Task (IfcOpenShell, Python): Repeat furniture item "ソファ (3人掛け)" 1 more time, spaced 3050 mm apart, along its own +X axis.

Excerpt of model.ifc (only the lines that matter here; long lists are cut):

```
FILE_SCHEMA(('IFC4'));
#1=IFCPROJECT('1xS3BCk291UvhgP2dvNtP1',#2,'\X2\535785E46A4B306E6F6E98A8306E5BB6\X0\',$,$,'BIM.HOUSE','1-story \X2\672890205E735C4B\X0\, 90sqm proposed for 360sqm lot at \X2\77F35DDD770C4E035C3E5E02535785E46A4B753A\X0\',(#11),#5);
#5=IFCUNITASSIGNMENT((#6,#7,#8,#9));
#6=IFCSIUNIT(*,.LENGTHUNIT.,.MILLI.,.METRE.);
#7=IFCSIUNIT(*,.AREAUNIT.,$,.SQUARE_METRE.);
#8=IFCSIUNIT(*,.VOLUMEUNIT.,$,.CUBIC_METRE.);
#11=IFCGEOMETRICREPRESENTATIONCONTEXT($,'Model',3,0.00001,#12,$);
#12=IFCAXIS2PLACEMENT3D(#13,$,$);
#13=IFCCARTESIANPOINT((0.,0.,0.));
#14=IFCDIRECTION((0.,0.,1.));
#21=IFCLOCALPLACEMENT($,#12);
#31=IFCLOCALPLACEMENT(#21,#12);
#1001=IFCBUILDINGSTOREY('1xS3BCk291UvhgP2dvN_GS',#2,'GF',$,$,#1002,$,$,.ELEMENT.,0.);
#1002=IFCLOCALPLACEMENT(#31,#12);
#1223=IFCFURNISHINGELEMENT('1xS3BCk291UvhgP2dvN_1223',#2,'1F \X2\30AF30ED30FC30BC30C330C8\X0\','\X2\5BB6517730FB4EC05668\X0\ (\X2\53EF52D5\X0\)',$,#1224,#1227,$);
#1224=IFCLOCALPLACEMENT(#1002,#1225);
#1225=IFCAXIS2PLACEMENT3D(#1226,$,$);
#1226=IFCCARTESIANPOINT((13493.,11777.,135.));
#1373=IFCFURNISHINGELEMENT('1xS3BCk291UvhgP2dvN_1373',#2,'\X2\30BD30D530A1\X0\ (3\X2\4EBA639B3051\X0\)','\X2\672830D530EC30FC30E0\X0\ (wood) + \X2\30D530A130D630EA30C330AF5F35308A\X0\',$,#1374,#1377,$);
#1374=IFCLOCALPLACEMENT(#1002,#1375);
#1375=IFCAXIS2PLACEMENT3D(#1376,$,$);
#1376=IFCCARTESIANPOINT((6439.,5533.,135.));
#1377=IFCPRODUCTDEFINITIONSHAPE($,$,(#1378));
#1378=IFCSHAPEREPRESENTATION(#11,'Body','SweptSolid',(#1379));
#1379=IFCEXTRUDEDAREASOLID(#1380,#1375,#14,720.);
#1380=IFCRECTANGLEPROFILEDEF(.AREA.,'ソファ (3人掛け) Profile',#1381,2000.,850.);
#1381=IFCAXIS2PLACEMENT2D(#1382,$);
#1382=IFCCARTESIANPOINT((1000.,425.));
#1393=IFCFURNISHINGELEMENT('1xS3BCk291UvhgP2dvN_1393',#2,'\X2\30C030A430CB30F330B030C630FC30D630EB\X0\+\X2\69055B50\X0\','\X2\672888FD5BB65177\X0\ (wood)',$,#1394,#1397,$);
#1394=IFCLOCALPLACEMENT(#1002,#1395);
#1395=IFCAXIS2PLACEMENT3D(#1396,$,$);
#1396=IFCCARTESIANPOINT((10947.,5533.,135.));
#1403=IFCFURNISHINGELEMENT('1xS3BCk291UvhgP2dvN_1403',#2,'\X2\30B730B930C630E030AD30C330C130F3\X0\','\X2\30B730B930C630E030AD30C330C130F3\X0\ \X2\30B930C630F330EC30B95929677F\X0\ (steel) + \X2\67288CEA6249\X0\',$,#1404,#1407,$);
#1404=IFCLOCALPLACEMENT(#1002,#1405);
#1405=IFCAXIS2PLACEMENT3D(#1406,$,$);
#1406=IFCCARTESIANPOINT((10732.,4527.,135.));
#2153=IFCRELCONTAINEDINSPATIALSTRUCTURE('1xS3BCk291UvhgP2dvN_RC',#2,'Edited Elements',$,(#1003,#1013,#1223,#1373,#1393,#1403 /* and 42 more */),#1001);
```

```python
import ifcopenshell
import ifcopenshell.api.geometry
import ifcopenshell.api.root
import ifcopenshell.util.element
import ifcopenshell.util.placement
import ifcopenshell.util.unit

model = ifcopenshell.open("model.ifc")
unit_scale = ifcopenshell.util.unit.calculate_unit_scale(model)


def reuse_history(source, copy):
    """copy_class also copies each property set's owner history, people and application; keep the originals."""
    for rel in copy.IsDefinedBy:
        if rel.is_a("IfcRelDefinesByProperties") and (history := rel.RelatingPropertyDefinition.OwnerHistory):
            rel.RelatingPropertyDefinition.OwnerHistory = source.OwnerHistory
            ifcopenshell.util.element.remove_deep2(model, history)


source = model.by_guid("1xS3BCk291UvhgP2dvN_1373")
base = ifcopenshell.util.placement.get_local_placement(source.ObjectPlacement)
step = base[:3, 0] * 3.05 / unit_scale

for i in range(1, 2):
    copy = ifcopenshell.api.root.copy_class(model, product=source)
    copy.Representation = ifcopenshell.util.element.copy_deep(
        model, source.Representation, exclude=["IfcGeometricRepresentationContext", "IfcRepresentationMap"]
    )
    reuse_history(source, copy)
    matrix = base.copy()
    matrix[:3, 3] += i * step
    print("added at", matrix[:3, 3].round(3) + 0.0)
    ifcopenshell.api.geometry.edit_object_placement(model, product=copy, matrix=matrix, is_si=False)

model.write("model-out.ifc")
```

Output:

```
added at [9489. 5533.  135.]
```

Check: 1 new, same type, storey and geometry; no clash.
